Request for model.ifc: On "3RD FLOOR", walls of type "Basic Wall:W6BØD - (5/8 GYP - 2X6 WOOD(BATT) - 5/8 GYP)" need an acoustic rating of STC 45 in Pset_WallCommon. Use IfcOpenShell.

First a look at what the model holds.

```python
import ifcopenshell
import ifcopenshell.util.element

model = ifcopenshell.open("model.ifc")
print(model.schema)
storey = next(s for s in model.by_type("IfcBuildingStorey") if s.Name == "3RD FLOOR")
walls = [e for e in ifcopenshell.util.element.get_decomposition(storey) if e.is_a("IfcWall")]
seen = {}
for e in walls:
    element_type = ifcopenshell.util.element.get_type(e)
    key = (element_type.Name if element_type != e and element_type else None, ifcopenshell.util.element.get_pset(e, "Pset_WallCommon", "AcousticRating"))
    seen[key] = seen.get(key, 0) + 1
for (name, value), count in sorted(seen.items(), key=str):
    print(count, "x", name, "|", value)
```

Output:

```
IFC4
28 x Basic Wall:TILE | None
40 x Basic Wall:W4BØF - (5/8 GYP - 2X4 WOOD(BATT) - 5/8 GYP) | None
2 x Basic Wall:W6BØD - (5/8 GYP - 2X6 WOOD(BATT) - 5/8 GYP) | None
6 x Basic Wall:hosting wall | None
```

```python
import ifcopenshell
import ifcopenshell.api.pset
import ifcopenshell.util.element

model = ifcopenshell.open("model.ifc")

storey = next(s for s in model.by_type("IfcBuildingStorey") if s.Name == "3RD FLOOR")
walls = [e for e in ifcopenshell.util.element.get_decomposition(storey) if e.is_a("IfcWall")]

count = 0
for e in walls:
    element_type = ifcopenshell.util.element.get_type(e)
    if element_type in (None, e) or element_type.Name != "Basic Wall:W6BØD - (5/8 GYP - 2X6 WOOD(BATT) - 5/8 GYP)":
        continue
    # add_pset returns the element's existing set when there is one.
    pset = ifcopenshell.api.pset.add_pset(model, product=e, name="Pset_WallCommon")
    ifcopenshell.api.pset.edit_pset(model, pset=pset, properties={"AcousticRating": "STC 45"})
    count += 1

print(count, "walls updated")

model.write("model_edited.ifc")
```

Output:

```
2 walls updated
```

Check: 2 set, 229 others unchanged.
